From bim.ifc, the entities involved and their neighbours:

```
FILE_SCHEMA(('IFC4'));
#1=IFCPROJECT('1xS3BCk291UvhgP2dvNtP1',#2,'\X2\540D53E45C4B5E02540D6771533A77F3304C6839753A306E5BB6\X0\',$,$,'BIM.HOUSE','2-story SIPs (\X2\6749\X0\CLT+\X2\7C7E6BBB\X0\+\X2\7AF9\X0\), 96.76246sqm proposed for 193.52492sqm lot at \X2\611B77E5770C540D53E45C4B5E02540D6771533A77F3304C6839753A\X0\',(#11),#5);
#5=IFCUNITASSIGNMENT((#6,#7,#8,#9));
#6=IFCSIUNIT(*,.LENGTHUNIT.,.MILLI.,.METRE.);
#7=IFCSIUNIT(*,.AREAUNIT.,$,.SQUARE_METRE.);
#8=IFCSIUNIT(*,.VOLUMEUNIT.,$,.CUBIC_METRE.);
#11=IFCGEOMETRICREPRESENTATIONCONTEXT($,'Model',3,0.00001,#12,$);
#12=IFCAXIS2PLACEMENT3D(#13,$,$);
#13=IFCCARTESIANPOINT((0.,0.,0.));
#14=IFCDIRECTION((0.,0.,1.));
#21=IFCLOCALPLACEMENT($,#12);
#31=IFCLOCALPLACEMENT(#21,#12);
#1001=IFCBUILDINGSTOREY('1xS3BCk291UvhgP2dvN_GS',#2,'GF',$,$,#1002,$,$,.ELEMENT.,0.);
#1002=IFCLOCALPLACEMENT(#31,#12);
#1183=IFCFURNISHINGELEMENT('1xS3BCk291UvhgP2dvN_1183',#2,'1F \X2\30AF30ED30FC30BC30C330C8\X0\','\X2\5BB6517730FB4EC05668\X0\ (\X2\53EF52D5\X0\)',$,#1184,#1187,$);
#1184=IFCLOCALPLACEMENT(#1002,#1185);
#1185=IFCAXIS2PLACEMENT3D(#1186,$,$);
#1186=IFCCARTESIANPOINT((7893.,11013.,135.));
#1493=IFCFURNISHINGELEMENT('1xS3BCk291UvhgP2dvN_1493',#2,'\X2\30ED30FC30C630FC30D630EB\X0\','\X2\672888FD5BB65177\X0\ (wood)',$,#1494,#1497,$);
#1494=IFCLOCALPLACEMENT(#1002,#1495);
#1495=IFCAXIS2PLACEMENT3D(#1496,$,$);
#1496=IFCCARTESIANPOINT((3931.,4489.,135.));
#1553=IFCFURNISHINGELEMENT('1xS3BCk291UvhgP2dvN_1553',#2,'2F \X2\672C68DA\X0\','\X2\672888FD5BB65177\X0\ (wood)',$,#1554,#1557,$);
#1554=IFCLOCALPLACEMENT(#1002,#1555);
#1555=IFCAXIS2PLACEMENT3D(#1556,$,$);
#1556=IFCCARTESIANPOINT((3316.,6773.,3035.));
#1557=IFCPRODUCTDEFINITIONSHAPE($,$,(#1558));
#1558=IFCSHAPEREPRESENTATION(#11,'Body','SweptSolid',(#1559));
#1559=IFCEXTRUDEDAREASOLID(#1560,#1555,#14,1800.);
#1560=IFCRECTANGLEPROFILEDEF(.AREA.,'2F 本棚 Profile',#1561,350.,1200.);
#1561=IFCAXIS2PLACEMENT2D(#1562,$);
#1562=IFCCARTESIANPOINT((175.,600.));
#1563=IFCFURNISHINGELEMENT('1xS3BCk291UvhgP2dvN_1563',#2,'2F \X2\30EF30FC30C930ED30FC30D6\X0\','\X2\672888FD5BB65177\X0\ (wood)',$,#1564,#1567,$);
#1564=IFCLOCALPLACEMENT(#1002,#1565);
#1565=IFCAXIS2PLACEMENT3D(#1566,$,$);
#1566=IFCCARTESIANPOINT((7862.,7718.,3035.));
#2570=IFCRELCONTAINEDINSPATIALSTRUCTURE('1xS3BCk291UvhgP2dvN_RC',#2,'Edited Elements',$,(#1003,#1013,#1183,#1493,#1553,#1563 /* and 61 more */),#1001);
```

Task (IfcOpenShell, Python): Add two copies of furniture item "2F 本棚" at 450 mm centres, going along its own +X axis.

```python
import ifcopenshell
import ifcopenshell.api.geometry
import ifcopenshell.api.root
import ifcopenshell.util.element
import ifcopenshell.util.placement
import ifcopenshell.util.unit

model = ifcopenshell.open("bim.ifc")
unit_scale = ifcopenshell.util.unit.calculate_unit_scale(model)


def reuse_history(source, copy):
    """copy_class also copies each property set's owner history, people and application; keep the originals."""
    for rel in copy.IsDefinedBy:
        if rel.is_a("IfcRelDefinesByProperties") and (history := rel.RelatingPropertyDefinition.OwnerHistory):
            rel.RelatingPropertyDefinition.OwnerHistory = source.OwnerHistory
            ifcopenshell.util.element.remove_deep2(model, history)


source = model.by_guid("1xS3BCk291UvhgP2dvN_1553")
base = ifcopenshell.util.placement.get_local_placement(source.ObjectPlacement)
step = base[:3, 0] * 0.45 / unit_scale

for i in range(1, 3):
    copy = ifcopenshell.api.root.copy_class(model, product=source)
    copy.Representation = ifcopenshell.util.element.copy_deep(
        model, source.Representation, exclude=["IfcGeometricRepresentationContext", "IfcRepresentationMap"]
    )
    reuse_history(source, copy)
    matrix = base.copy()
    matrix[:3, 3] += i * step
    print("added at", matrix[:3, 3].round(3) + 0.0)
    ifcopenshell.api.geometry.edit_object_placement(model, product=copy, matrix=matrix, is_si=False)

model.write("bim-out.ifc")
```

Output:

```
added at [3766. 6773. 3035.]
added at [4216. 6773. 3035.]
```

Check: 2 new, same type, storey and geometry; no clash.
